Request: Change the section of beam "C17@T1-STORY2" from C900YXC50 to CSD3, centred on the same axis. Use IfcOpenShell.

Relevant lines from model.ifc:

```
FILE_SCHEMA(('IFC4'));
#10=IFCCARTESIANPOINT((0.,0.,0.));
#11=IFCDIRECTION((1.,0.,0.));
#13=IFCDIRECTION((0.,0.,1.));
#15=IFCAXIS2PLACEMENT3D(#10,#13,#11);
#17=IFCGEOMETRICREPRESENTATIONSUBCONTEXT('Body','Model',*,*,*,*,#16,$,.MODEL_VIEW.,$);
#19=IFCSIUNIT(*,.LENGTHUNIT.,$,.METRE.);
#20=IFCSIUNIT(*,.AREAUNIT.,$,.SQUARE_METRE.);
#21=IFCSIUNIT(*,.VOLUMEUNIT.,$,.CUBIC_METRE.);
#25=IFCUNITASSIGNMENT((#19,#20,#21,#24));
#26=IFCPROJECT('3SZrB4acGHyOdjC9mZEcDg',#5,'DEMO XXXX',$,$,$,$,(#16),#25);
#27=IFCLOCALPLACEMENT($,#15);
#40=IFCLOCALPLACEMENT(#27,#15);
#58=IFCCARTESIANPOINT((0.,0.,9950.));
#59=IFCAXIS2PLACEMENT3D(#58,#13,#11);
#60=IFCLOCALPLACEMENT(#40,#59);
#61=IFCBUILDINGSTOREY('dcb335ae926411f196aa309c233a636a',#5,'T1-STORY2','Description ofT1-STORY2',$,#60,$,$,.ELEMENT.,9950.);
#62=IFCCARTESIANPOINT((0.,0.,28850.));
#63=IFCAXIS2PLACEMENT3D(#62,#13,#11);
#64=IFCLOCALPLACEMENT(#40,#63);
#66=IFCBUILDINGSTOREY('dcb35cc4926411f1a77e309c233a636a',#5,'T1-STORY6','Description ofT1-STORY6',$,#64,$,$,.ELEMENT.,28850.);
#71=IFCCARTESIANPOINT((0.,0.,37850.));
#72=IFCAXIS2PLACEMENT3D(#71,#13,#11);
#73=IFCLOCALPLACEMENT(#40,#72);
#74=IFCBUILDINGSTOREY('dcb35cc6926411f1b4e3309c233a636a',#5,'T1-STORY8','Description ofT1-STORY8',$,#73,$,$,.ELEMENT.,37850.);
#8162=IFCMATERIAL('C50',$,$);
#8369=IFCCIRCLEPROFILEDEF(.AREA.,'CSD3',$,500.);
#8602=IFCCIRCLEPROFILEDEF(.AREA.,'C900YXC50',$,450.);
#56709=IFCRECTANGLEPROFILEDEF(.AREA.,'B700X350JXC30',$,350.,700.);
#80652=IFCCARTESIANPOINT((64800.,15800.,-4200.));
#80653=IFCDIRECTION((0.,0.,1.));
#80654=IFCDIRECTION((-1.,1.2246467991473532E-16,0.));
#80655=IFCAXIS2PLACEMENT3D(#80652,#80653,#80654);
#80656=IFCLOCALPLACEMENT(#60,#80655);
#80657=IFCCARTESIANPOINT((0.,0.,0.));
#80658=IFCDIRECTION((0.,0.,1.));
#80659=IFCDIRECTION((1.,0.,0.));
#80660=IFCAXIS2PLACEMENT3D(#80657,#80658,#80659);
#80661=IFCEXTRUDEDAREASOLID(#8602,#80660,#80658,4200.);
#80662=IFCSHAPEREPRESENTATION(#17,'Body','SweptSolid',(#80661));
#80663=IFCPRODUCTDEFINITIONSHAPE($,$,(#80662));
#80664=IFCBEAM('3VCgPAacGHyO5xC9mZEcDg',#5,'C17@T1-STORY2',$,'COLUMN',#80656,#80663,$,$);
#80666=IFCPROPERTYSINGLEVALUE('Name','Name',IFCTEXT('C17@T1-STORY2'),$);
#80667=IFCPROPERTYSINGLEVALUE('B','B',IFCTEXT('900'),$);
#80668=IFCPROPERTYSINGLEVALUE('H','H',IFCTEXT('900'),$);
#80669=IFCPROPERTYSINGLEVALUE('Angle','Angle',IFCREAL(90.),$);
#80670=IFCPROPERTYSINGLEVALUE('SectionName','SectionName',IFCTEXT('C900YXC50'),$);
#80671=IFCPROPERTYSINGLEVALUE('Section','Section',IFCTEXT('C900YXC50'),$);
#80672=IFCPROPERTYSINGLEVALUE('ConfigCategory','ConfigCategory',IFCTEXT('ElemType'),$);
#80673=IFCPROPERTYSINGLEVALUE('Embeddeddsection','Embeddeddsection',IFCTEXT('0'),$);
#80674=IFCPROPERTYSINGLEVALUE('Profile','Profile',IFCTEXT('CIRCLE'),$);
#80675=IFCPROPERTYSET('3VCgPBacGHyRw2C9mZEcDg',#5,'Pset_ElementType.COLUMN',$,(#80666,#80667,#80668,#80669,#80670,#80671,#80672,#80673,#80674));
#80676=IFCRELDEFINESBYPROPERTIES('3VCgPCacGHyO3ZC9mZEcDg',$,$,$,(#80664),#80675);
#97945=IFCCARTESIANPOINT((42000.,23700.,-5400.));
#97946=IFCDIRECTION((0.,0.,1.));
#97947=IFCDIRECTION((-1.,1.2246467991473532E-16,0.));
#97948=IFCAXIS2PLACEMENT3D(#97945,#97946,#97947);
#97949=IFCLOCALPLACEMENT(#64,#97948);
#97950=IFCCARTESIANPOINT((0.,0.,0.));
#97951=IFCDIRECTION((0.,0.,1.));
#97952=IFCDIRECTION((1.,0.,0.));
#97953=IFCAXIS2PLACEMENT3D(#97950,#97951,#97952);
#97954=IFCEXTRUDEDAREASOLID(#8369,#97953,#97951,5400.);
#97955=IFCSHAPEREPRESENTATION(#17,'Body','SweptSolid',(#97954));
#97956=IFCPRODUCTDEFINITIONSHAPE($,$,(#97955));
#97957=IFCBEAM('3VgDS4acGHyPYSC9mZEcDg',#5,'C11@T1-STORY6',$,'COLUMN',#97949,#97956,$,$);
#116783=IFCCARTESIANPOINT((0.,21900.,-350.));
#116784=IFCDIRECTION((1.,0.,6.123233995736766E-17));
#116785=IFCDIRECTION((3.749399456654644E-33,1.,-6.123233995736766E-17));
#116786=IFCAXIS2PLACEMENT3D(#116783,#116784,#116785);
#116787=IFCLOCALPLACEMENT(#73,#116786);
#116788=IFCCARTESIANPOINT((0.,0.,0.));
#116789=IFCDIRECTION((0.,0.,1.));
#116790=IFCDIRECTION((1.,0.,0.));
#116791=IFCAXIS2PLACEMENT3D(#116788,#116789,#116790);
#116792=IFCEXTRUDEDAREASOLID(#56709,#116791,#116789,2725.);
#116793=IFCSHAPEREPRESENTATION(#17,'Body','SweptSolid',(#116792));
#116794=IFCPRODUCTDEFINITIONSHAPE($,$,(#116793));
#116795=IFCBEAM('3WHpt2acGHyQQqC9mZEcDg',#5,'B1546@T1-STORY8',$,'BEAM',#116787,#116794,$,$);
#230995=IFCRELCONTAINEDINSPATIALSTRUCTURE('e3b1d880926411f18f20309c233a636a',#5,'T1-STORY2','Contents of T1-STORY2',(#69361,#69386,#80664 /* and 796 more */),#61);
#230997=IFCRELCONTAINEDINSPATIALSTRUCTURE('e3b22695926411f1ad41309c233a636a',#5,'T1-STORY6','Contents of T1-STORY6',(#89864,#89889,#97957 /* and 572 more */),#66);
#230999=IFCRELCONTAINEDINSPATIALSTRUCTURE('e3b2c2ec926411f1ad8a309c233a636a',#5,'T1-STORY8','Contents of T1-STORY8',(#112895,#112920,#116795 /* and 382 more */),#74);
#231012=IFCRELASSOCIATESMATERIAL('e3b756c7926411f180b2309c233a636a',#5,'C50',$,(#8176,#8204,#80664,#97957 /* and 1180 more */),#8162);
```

```python
import ifcopenshell
import ifcopenshell.api.pset
import ifcopenshell.util.element
import ifcopenshell.util.representation

model = ifcopenshell.open("model.ifc")

member = model.by_guid("3VCgPAacGHyO5xC9mZEcDg")
source = next(p for p in model.by_type("IfcCircleProfileDef") if p.ProfileName == "CSD3")

body = ifcopenshell.util.representation.get_representation(member, "Model", "Body")
solid = body.Items[0]
old_profile = solid.SweptArea

# Copy the section's sizes but keep this member's own profile position.
profile = ifcopenshell.util.element.copy(model, source)
profile.Position = old_profile.Position
solid.SweptArea = profile
if not model.get_total_inverses(old_profile):
    ifcopenshell.util.element.remove_deep2(model, old_profile)
pset = model.by_id(ifcopenshell.util.element.get_pset(member, "Pset_ElementType.COLUMN", should_inherit=False)["id"])
ifcopenshell.api.pset.edit_pset(model, pset=pset, properties={"SectionName": "CSD3"})
pset = model.by_id(ifcopenshell.util.element.get_pset(member, "Pset_ElementType.COLUMN", should_inherit=False)["id"])
ifcopenshell.api.pset.edit_pset(model, pset=pset, properties={"Section": "CSD3"})

print(solid.SweptArea)

model.write("model_rev.ifc")
```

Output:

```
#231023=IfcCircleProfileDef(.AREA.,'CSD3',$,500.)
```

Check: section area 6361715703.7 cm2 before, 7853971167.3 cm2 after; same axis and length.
